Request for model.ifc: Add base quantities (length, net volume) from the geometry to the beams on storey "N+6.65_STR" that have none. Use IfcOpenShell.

First a look at what the model holds.

```python
import ifcopenshell
import ifcopenshell.util.element
import ifcopenshell.util.unit

model = ifcopenshell.open("model.ifc")
print(model.schema)
for unit_type in ("LENGTHUNIT", "AREAUNIT", "VOLUMEUNIT"):
    print(unit_type, ifcopenshell.util.unit.calculate_unit_scale(model, unit_type))
storey = next(s for s in model.by_type("IfcBuildingStorey") if s.Name == "N+6.65_STR")
beams = [e for e in ifcopenshell.util.element.get_decomposition(storey) if e.is_a("IfcBeam")]
for e in sorted(beams, key=lambda e: e.id()):
    print(e.id(), e.is_a(), e.Name, list(ifcopenshell.util.element.get_psets(e, qtos_only=True)), sep=" | ")
```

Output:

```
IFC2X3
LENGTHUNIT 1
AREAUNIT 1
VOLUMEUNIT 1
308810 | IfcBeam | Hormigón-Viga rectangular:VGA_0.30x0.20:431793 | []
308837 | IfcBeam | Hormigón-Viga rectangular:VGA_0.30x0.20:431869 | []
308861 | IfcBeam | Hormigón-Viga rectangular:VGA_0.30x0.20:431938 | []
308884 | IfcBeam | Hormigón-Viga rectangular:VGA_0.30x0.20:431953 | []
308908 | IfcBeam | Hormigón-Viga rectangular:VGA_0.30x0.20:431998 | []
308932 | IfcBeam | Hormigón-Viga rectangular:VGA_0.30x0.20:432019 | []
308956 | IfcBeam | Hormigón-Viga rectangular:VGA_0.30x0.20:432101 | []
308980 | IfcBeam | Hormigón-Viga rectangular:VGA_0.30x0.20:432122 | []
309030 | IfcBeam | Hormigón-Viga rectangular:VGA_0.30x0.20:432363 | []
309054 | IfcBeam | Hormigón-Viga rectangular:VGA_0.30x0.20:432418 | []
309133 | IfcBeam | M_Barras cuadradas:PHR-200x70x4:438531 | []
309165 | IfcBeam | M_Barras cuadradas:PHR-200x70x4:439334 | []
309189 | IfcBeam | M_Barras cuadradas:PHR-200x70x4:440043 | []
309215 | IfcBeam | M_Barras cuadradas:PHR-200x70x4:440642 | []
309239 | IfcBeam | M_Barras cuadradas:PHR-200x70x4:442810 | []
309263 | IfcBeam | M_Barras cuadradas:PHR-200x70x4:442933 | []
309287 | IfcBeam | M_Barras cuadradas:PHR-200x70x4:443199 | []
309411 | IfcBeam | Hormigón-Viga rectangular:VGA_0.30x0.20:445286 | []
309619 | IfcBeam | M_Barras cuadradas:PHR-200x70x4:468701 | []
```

```python
import ifcopenshell
import ifcopenshell.api.pset
import ifcopenshell.geom
import ifcopenshell.util.element
import ifcopenshell.util.shape
import ifcopenshell.util.unit

model = ifcopenshell.open("model.ifc")
unit_scale = ifcopenshell.util.unit.calculate_unit_scale(model)
volume_scale = ifcopenshell.util.unit.calculate_unit_scale(model, "VOLUMEUNIT")
settings = ifcopenshell.geom.settings()

storey = next(s for s in model.by_type("IfcBuildingStorey") if s.Name == "N+6.65_STR")
beams = [e for e in ifcopenshell.util.element.get_decomposition(storey) if e.is_a("IfcBeam")]

for e in sorted(beams, key=lambda e: e.id()):
    if ifcopenshell.util.element.get_psets(e, qtos_only=True, should_inherit=False):
        continue
    # Geometry comes back in metres, in the element's own axes.
    shape = ifcopenshell.geom.create_shape(settings, e)
    values = {
        "Length": ifcopenshell.util.shape.get_max_xyz(shape.geometry) / unit_scale,
        "NetVolume": ifcopenshell.util.shape.get_volume(shape.geometry) / volume_scale,
    }
    qto = ifcopenshell.api.pset.add_qto(model, product=e, name="BaseQuantities")
    ifcopenshell.api.pset.edit_qto(model, qto=qto, properties=values)
    print(e.id(), {k: round(v, 3) for k, v in values.items()})

model.write("model_v2.ifc")
```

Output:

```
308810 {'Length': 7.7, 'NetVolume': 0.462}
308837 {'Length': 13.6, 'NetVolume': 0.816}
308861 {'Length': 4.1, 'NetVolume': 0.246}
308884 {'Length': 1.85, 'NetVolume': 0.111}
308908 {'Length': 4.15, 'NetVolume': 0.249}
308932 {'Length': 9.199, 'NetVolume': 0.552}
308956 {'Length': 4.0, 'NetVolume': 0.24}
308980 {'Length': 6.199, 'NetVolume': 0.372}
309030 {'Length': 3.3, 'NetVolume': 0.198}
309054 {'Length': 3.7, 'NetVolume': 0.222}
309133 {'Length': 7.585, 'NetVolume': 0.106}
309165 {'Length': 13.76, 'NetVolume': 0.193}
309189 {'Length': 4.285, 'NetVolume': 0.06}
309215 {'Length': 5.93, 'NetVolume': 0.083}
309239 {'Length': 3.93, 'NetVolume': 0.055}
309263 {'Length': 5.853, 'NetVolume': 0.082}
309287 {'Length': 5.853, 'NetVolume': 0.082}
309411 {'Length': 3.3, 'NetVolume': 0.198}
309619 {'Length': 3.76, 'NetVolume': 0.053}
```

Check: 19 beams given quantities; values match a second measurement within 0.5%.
